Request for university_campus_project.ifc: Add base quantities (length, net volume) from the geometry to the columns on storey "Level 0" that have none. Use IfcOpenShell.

First a look at what the model holds.

```python
import ifcopenshell
import ifcopenshell.util.element
import ifcopenshell.util.unit

model = ifcopenshell.open("university_campus_project.ifc")
print(model.schema)
for unit_type in ("LENGTHUNIT", "AREAUNIT", "VOLUMEUNIT"):
    print(unit_type, ifcopenshell.util.unit.calculate_unit_scale(model, unit_type))
storey = next(s for s in model.by_type("IfcBuildingStorey") if s.Name == "Level 0")
columns = [e for e in ifcopenshell.util.element.get_decomposition(storey) if e.is_a("IfcColumn")]
for e in sorted(columns, key=lambda e: e.id()):
    print(e.id(), e.is_a(), e.Name, list(ifcopenshell.util.element.get_psets(e, qtos_only=True)), sep=" | ")
```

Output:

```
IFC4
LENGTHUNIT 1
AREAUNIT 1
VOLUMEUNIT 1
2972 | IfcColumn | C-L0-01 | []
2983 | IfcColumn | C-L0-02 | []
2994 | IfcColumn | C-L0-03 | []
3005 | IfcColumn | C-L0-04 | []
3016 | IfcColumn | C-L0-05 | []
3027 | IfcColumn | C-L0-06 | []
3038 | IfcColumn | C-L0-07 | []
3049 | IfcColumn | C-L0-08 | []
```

```python
import ifcopenshell
import ifcopenshell.api.pset
import ifcopenshell.geom
import ifcopenshell.util.element
import ifcopenshell.util.shape
import ifcopenshell.util.unit

model = ifcopenshell.open("university_campus_project.ifc")
unit_scale = ifcopenshell.util.unit.calculate_unit_scale(model)
volume_scale = ifcopenshell.util.unit.calculate_unit_scale(model, "VOLUMEUNIT")
settings = ifcopenshell.geom.settings()

storey = next(s for s in model.by_type("IfcBuildingStorey") if s.Name == "Level 0")
columns = [e for e in ifcopenshell.util.element.get_decomposition(storey) if e.is_a("IfcColumn")]

for e in sorted(columns, key=lambda e: e.id()):
    if ifcopenshell.util.element.get_psets(e, qtos_only=True, should_inherit=False):
        continue
    # Geometry comes back in metres, in the element's own axes.
    shape = ifcopenshell.geom.create_shape(settings, e)
    values = {
        "Length": ifcopenshell.util.shape.get_z(shape.geometry) / unit_scale,
        "NetVolume": ifcopenshell.util.shape.get_volume(shape.geometry) / volume_scale,
    }
    qto = ifcopenshell.api.pset.add_qto(model, product=e, name="Qto_ColumnBaseQuantities")
    ifcopenshell.api.pset.edit_qto(model, qto=qto, properties=values)
    print(e.id(), {k: round(v, 3) for k, v in values.items()})

model.write("university_campus_project_updated.ifc")
```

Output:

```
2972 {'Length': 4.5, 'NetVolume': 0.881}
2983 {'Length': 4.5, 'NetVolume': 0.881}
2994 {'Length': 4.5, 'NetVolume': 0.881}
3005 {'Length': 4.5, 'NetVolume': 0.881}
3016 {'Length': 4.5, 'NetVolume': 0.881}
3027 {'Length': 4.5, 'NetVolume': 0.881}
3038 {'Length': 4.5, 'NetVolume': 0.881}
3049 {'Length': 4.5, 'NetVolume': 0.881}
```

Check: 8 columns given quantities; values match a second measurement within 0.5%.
